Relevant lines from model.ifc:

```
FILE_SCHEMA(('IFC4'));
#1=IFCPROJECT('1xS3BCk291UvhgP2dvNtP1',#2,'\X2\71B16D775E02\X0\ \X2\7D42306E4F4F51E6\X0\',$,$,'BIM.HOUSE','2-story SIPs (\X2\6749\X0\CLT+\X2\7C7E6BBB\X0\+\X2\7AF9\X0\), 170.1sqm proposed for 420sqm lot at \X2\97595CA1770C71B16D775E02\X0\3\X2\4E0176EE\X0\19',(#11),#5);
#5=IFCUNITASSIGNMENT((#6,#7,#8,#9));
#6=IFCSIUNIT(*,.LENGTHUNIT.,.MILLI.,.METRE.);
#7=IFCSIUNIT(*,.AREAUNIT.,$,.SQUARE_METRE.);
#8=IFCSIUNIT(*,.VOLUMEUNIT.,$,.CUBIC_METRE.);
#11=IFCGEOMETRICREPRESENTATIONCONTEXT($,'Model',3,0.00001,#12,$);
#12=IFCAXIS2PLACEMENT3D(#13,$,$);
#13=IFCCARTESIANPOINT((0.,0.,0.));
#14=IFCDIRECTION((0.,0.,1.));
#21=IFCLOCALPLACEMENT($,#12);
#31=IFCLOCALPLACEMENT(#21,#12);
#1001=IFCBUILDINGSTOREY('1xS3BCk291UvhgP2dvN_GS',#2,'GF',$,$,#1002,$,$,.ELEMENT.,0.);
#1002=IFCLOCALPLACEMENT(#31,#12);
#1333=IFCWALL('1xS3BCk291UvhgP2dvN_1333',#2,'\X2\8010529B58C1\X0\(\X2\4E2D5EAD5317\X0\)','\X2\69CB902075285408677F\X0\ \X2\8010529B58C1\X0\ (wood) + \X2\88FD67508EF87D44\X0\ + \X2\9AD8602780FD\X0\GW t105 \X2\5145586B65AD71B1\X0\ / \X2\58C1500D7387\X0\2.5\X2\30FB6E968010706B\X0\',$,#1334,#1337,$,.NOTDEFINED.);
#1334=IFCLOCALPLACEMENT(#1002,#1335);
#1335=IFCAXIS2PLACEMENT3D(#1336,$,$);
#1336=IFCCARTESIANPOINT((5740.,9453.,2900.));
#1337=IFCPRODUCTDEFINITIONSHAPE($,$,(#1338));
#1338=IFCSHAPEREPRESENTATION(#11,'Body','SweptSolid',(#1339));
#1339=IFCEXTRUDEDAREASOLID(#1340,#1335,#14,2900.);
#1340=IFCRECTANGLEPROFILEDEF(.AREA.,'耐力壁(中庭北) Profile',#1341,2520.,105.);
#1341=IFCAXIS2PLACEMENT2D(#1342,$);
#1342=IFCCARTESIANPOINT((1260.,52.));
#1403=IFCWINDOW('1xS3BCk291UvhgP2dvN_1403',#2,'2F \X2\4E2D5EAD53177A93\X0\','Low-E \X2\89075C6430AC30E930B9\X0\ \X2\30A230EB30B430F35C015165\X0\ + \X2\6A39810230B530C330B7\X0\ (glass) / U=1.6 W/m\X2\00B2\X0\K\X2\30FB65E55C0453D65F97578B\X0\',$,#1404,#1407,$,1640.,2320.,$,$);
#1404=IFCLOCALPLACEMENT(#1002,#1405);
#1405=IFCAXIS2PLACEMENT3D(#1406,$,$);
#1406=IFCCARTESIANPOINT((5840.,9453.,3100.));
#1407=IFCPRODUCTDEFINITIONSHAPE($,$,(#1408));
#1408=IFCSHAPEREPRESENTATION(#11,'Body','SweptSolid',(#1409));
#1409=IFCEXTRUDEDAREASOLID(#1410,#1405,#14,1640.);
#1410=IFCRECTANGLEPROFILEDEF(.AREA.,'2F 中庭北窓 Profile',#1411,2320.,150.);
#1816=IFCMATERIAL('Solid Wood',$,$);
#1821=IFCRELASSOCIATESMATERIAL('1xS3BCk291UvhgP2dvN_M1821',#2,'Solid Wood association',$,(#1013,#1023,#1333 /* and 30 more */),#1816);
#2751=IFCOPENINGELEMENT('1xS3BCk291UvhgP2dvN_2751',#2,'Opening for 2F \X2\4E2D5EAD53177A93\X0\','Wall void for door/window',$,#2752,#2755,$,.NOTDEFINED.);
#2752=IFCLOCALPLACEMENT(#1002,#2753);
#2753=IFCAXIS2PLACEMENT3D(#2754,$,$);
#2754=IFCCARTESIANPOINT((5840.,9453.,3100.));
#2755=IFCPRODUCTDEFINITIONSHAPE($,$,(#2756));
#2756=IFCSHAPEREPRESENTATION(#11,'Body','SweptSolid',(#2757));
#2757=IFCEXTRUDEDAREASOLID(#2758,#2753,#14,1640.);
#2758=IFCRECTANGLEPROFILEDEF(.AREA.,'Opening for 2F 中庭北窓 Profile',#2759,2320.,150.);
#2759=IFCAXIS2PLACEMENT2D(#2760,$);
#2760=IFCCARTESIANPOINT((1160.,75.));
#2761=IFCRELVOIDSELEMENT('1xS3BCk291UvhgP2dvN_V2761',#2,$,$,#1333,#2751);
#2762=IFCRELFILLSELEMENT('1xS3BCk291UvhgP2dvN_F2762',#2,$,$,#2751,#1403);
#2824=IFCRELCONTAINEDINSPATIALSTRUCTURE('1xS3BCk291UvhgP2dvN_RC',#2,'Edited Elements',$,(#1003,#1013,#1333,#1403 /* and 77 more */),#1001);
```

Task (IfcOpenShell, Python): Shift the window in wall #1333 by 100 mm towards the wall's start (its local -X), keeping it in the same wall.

```python
import ifcopenshell
import ifcopenshell.api.geometry
import ifcopenshell.util.placement
import ifcopenshell.util.unit

model = ifcopenshell.open("model.ifc")
unit_scale = ifcopenshell.util.unit.calculate_unit_scale(model)

window = model.by_guid("1xS3BCk291UvhgP2dvN_1403")
opening = window.FillsVoids[0].RelatingOpeningElement
wall = opening.VoidsElements[0].RelatingBuildingElement

wall_matrix = ifcopenshell.util.placement.get_local_placement(wall.ObjectPlacement)
shift = wall_matrix[:3, 0] * -0.1 / unit_scale
before = ifcopenshell.util.placement.get_local_placement(window.ObjectPlacement)[:3, 3].copy()

# The window is not placed relative to its opening, so move both.
for product in (opening, window):
    matrix = ifcopenshell.util.placement.get_local_placement(product.ObjectPlacement)
    matrix[:3, 3] += shift
    ifcopenshell.api.geometry.edit_object_placement(model, product=product, matrix=matrix, is_si=False)

after = ifcopenshell.util.placement.get_local_placement(window.ObjectPlacement)[:3, 3]
print("window moved by", (after - before).round(3) + 0.0)

model.write("model_rev.ifc")
```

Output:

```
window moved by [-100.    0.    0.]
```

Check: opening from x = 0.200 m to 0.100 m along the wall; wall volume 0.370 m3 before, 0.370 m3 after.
